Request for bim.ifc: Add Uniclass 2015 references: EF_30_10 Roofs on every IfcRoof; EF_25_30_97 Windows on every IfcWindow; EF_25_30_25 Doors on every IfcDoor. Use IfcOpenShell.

First a look at what the model holds.

```python
import ifcopenshell

model = ifcopenshell.open("bim.ifc")
print(model.schema)
print("classifications:", [c.Name for c in model.by_type("IfcClassification")])
for ifc_class in ("IfcDoor", "IfcRoof", "IfcStair", "IfcWall", "IfcWindow"):
    print(ifc_class, len(model.by_type(ifc_class)))
```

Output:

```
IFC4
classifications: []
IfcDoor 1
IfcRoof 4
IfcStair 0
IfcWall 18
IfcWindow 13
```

```python
import ifcopenshell
import ifcopenshell.api.classification

model = ifcopenshell.open("bim.ifc")

system = ifcopenshell.api.classification.add_classification(model, classification="Uniclass 2015")

codes = {
    "IfcRoof": ("EF_30_10", "Roofs"),
    "IfcWindow": ("EF_25_30_97", "Windows"),
    "IfcDoor": ("EF_25_30_25", "Doors"),
}
for ifc_class, (code, name) in codes.items():
    products = model.by_type(ifc_class)
    ifcopenshell.api.classification.add_reference(
        model, products=products, classification=system, identification=code, name=name
    )
    print(code, len(products))

model.write("bim_rev.ifc")
```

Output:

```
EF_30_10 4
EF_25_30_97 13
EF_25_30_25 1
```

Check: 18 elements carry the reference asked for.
